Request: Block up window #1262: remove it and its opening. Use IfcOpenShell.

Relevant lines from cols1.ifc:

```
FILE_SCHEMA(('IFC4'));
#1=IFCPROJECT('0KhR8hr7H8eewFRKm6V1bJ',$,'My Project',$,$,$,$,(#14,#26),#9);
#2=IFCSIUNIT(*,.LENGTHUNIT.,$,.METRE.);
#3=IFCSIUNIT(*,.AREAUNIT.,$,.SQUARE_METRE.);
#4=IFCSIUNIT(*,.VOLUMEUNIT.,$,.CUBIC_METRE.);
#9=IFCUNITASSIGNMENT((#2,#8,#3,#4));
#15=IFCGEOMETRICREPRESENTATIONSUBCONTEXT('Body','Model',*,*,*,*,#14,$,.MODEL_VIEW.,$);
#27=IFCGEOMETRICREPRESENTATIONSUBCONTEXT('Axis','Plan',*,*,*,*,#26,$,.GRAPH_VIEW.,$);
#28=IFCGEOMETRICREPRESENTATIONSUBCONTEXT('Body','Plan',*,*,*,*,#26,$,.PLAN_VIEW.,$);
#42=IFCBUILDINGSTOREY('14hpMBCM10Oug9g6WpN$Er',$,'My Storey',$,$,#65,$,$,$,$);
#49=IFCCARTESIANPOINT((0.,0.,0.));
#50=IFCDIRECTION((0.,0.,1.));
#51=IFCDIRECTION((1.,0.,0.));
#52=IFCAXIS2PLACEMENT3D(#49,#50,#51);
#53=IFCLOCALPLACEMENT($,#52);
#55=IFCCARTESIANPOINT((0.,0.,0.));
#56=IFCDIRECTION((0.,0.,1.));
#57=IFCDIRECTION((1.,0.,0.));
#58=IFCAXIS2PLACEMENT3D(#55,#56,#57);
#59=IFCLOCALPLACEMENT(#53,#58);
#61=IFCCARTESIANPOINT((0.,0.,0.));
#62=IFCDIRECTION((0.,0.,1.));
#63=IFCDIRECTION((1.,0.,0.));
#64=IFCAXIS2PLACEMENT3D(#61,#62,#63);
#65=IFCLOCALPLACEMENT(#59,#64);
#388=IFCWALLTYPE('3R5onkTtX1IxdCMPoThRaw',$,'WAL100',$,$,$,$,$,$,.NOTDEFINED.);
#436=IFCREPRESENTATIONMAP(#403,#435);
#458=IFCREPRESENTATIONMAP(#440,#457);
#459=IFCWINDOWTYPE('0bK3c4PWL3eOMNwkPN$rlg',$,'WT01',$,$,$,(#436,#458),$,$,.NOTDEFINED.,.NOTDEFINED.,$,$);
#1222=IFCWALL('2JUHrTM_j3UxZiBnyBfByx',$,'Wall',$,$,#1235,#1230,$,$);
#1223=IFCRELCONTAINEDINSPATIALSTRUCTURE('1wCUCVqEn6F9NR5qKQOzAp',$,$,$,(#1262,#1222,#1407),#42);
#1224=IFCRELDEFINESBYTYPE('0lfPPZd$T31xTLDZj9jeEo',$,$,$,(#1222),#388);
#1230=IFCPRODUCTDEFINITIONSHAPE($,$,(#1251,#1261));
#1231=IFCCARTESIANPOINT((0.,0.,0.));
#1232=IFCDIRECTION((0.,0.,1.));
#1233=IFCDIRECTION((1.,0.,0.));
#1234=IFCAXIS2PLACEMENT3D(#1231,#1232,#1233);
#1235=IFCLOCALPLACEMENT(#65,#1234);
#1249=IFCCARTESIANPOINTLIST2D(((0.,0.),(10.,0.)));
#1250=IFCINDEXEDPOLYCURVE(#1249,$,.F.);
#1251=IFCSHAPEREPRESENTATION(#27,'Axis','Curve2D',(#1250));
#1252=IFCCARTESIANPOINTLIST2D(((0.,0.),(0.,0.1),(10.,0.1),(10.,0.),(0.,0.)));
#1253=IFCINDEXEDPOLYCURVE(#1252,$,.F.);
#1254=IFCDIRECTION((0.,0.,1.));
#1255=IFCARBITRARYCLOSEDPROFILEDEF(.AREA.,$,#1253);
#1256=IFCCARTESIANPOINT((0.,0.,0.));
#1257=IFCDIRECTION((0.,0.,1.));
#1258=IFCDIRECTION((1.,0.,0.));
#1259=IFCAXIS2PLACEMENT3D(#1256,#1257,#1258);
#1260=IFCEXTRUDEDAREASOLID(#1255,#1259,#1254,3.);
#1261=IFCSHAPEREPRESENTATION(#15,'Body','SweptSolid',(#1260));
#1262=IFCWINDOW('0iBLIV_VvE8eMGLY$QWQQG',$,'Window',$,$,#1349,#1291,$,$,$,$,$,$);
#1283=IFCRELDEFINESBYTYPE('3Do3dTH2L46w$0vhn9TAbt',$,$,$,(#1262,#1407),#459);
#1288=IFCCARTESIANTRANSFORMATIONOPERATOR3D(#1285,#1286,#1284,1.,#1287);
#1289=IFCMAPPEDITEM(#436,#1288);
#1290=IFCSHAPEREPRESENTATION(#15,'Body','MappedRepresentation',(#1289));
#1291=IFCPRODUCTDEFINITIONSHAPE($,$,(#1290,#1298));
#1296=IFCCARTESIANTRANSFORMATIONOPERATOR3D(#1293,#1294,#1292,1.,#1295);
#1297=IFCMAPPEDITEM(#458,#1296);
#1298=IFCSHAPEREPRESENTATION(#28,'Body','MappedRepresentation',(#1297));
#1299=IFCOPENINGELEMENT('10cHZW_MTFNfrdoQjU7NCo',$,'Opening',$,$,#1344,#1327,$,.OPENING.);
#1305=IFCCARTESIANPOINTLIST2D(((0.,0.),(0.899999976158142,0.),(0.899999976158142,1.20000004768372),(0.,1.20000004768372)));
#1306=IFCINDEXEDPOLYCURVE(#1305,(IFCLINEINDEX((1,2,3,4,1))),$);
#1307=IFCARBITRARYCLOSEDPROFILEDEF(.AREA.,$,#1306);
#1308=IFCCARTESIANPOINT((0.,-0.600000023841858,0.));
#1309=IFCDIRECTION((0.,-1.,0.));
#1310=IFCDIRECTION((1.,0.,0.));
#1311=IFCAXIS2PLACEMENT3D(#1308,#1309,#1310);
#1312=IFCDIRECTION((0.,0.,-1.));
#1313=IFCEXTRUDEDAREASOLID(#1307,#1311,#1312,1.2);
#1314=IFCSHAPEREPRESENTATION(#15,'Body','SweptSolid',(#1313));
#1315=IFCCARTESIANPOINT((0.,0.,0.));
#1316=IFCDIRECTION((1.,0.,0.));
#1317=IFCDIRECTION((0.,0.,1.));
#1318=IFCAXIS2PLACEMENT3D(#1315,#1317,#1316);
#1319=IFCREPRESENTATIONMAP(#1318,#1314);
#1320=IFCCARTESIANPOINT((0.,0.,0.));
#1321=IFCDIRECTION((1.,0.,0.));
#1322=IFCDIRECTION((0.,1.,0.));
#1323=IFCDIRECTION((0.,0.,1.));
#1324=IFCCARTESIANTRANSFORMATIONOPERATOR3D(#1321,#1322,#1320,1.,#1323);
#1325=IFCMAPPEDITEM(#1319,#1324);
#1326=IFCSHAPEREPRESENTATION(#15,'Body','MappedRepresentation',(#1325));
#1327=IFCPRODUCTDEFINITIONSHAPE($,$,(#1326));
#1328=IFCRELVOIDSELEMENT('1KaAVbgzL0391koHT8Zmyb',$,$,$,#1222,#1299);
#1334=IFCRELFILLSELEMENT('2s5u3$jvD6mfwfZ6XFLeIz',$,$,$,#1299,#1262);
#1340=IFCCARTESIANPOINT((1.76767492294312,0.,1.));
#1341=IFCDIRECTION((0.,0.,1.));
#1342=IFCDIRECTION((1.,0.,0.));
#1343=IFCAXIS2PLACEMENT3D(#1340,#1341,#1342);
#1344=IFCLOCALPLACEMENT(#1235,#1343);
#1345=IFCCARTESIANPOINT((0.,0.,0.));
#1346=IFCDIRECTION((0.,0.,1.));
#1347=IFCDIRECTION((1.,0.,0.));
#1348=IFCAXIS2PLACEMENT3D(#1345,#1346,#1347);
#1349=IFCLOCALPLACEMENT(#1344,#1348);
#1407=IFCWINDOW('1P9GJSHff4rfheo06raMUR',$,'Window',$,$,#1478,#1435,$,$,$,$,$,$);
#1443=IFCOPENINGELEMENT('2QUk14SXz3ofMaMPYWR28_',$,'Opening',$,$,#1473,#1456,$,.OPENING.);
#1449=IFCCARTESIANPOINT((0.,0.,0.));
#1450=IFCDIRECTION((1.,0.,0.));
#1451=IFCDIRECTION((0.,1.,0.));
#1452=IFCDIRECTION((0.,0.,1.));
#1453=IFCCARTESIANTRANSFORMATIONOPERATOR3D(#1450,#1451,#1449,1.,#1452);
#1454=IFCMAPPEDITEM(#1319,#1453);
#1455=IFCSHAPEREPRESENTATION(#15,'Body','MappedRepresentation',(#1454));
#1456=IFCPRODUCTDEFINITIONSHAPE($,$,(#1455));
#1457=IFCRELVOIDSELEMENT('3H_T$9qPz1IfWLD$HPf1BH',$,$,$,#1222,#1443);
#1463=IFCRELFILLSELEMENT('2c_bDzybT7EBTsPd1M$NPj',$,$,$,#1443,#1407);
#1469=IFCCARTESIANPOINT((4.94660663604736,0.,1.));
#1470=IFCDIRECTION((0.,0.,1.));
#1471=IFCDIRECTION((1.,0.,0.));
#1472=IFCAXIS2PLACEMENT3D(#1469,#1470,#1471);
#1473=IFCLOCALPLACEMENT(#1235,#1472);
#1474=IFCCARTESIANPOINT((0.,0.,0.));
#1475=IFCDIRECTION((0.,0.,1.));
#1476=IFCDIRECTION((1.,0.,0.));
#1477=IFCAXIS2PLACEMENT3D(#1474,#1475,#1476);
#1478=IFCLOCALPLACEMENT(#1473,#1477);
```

```python
import ifcopenshell
import ifcopenshell.api.feature
import ifcopenshell.api.root
import ifcopenshell.geom
import ifcopenshell.util.shape

model = ifcopenshell.open("cols1.ifc")
settings = ifcopenshell.geom.settings()


def volume(element):
    """Net volume in cubic metres, openings subtracted."""
    shape = ifcopenshell.geom.create_shape(settings, element)
    return ifcopenshell.util.shape.get_volume(shape.geometry)


window = model.by_guid("0iBLIV_VvE8eMGLY$QWQQG")
opening = window.FillsVoids[0].RelatingOpeningElement
wall = opening.VoidsElements[0].RelatingBuildingElement
before = volume(wall)

ifcopenshell.api.root.remove_product(model, product=window)
ifcopenshell.api.feature.remove_feature(model, feature=opening)

after = volume(wall)

print(f"wall volume {before:.3f} -> {after:.3f} m3")

model.write("cols1_edited.ifc")
```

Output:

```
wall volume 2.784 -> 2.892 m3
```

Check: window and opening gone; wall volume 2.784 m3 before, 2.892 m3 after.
